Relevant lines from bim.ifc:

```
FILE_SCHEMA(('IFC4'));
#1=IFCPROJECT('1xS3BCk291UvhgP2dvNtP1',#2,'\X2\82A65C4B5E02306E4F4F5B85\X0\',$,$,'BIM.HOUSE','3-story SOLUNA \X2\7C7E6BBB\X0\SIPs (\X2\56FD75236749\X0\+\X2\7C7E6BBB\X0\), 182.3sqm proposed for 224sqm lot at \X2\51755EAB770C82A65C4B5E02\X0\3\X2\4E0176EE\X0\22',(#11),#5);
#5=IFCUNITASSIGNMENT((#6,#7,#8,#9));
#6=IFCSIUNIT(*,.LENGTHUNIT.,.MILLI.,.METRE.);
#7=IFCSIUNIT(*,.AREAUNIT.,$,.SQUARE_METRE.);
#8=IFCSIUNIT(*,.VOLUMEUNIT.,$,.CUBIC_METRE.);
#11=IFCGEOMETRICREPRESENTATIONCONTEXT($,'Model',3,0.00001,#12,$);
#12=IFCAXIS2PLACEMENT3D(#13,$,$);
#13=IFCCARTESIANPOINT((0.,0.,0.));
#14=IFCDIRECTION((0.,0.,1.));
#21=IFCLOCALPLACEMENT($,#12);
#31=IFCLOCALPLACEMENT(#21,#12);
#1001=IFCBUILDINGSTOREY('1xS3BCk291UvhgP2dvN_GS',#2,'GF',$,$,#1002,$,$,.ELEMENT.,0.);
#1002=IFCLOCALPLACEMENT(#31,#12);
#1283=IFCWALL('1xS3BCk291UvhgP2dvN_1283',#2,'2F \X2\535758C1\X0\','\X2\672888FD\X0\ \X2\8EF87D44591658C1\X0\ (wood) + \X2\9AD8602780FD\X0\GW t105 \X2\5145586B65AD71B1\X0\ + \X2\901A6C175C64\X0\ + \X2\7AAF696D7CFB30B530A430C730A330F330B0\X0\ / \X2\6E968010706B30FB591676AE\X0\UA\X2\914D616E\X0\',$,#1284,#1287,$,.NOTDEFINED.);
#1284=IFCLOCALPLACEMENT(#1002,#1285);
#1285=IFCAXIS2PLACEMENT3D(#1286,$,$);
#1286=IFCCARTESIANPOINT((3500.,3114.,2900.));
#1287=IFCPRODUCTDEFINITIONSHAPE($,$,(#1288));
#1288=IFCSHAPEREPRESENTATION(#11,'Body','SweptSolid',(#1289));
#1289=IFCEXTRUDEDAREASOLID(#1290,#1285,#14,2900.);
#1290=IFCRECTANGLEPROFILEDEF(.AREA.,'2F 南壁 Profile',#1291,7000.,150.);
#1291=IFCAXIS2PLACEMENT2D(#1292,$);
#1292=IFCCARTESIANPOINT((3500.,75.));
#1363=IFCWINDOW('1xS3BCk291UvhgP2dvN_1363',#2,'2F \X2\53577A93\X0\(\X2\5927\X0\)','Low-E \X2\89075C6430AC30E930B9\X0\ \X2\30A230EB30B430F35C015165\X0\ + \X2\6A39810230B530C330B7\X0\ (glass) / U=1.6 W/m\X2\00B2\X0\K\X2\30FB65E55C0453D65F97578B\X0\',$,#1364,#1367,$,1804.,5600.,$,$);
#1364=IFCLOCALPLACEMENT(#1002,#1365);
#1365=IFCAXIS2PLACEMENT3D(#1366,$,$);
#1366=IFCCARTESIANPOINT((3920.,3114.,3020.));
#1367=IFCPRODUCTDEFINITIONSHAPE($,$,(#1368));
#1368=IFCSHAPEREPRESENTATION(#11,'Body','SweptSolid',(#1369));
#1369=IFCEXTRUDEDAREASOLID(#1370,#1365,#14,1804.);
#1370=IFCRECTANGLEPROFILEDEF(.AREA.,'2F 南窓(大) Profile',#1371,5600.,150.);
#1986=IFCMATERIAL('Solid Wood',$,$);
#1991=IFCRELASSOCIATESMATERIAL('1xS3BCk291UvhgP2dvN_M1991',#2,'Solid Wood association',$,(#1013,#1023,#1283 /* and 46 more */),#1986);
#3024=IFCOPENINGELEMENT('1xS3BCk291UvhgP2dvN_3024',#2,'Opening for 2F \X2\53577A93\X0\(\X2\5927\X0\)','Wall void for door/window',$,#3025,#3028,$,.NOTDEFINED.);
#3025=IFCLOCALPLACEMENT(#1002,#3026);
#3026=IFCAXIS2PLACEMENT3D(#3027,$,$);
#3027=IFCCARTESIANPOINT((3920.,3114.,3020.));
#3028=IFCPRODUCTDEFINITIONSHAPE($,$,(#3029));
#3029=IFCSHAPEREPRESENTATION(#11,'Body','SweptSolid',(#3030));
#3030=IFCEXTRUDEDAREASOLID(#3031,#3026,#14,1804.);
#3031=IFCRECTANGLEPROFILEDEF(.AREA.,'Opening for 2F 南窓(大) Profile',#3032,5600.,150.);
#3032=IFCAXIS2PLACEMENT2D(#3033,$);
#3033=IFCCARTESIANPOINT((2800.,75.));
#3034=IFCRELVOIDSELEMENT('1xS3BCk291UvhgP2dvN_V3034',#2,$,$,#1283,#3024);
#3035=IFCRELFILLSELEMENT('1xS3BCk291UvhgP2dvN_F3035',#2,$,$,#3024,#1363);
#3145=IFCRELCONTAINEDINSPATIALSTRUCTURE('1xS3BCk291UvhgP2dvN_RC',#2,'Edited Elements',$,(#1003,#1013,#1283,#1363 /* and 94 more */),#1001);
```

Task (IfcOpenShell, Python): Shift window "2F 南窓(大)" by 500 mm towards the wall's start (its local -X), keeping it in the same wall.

```python
import ifcopenshell
import ifcopenshell.api.geometry
import ifcopenshell.util.placement

model = ifcopenshell.open("bim.ifc")

window = model.by_guid("1xS3BCk291UvhgP2dvN_1363")
opening = window.FillsVoids[0].RelatingOpeningElement
wall = opening.VoidsElements[0].RelatingBuildingElement

wall_matrix = ifcopenshell.util.placement.get_local_placement(wall.ObjectPlacement)
shift = wall_matrix[:3, 0] * -500.0
before = ifcopenshell.util.placement.get_local_placement(window.ObjectPlacement)[:3, 3].copy()

# The window is not placed relative to its opening, so move both.
for product in (opening, window):
    matrix = ifcopenshell.util.placement.get_local_placement(product.ObjectPlacement)
    matrix[:3, 3] += shift
    ifcopenshell.api.geometry.edit_object_placement(model, product=product, matrix=matrix, is_si=False)

after = ifcopenshell.util.placement.get_local_placement(window.ObjectPlacement)[:3, 3]
print("window moved by", (after - before).round(3) + 0.0)

model.write("bim-out.ifc")
```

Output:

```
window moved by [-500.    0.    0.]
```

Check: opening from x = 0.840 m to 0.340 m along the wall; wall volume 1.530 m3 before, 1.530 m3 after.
